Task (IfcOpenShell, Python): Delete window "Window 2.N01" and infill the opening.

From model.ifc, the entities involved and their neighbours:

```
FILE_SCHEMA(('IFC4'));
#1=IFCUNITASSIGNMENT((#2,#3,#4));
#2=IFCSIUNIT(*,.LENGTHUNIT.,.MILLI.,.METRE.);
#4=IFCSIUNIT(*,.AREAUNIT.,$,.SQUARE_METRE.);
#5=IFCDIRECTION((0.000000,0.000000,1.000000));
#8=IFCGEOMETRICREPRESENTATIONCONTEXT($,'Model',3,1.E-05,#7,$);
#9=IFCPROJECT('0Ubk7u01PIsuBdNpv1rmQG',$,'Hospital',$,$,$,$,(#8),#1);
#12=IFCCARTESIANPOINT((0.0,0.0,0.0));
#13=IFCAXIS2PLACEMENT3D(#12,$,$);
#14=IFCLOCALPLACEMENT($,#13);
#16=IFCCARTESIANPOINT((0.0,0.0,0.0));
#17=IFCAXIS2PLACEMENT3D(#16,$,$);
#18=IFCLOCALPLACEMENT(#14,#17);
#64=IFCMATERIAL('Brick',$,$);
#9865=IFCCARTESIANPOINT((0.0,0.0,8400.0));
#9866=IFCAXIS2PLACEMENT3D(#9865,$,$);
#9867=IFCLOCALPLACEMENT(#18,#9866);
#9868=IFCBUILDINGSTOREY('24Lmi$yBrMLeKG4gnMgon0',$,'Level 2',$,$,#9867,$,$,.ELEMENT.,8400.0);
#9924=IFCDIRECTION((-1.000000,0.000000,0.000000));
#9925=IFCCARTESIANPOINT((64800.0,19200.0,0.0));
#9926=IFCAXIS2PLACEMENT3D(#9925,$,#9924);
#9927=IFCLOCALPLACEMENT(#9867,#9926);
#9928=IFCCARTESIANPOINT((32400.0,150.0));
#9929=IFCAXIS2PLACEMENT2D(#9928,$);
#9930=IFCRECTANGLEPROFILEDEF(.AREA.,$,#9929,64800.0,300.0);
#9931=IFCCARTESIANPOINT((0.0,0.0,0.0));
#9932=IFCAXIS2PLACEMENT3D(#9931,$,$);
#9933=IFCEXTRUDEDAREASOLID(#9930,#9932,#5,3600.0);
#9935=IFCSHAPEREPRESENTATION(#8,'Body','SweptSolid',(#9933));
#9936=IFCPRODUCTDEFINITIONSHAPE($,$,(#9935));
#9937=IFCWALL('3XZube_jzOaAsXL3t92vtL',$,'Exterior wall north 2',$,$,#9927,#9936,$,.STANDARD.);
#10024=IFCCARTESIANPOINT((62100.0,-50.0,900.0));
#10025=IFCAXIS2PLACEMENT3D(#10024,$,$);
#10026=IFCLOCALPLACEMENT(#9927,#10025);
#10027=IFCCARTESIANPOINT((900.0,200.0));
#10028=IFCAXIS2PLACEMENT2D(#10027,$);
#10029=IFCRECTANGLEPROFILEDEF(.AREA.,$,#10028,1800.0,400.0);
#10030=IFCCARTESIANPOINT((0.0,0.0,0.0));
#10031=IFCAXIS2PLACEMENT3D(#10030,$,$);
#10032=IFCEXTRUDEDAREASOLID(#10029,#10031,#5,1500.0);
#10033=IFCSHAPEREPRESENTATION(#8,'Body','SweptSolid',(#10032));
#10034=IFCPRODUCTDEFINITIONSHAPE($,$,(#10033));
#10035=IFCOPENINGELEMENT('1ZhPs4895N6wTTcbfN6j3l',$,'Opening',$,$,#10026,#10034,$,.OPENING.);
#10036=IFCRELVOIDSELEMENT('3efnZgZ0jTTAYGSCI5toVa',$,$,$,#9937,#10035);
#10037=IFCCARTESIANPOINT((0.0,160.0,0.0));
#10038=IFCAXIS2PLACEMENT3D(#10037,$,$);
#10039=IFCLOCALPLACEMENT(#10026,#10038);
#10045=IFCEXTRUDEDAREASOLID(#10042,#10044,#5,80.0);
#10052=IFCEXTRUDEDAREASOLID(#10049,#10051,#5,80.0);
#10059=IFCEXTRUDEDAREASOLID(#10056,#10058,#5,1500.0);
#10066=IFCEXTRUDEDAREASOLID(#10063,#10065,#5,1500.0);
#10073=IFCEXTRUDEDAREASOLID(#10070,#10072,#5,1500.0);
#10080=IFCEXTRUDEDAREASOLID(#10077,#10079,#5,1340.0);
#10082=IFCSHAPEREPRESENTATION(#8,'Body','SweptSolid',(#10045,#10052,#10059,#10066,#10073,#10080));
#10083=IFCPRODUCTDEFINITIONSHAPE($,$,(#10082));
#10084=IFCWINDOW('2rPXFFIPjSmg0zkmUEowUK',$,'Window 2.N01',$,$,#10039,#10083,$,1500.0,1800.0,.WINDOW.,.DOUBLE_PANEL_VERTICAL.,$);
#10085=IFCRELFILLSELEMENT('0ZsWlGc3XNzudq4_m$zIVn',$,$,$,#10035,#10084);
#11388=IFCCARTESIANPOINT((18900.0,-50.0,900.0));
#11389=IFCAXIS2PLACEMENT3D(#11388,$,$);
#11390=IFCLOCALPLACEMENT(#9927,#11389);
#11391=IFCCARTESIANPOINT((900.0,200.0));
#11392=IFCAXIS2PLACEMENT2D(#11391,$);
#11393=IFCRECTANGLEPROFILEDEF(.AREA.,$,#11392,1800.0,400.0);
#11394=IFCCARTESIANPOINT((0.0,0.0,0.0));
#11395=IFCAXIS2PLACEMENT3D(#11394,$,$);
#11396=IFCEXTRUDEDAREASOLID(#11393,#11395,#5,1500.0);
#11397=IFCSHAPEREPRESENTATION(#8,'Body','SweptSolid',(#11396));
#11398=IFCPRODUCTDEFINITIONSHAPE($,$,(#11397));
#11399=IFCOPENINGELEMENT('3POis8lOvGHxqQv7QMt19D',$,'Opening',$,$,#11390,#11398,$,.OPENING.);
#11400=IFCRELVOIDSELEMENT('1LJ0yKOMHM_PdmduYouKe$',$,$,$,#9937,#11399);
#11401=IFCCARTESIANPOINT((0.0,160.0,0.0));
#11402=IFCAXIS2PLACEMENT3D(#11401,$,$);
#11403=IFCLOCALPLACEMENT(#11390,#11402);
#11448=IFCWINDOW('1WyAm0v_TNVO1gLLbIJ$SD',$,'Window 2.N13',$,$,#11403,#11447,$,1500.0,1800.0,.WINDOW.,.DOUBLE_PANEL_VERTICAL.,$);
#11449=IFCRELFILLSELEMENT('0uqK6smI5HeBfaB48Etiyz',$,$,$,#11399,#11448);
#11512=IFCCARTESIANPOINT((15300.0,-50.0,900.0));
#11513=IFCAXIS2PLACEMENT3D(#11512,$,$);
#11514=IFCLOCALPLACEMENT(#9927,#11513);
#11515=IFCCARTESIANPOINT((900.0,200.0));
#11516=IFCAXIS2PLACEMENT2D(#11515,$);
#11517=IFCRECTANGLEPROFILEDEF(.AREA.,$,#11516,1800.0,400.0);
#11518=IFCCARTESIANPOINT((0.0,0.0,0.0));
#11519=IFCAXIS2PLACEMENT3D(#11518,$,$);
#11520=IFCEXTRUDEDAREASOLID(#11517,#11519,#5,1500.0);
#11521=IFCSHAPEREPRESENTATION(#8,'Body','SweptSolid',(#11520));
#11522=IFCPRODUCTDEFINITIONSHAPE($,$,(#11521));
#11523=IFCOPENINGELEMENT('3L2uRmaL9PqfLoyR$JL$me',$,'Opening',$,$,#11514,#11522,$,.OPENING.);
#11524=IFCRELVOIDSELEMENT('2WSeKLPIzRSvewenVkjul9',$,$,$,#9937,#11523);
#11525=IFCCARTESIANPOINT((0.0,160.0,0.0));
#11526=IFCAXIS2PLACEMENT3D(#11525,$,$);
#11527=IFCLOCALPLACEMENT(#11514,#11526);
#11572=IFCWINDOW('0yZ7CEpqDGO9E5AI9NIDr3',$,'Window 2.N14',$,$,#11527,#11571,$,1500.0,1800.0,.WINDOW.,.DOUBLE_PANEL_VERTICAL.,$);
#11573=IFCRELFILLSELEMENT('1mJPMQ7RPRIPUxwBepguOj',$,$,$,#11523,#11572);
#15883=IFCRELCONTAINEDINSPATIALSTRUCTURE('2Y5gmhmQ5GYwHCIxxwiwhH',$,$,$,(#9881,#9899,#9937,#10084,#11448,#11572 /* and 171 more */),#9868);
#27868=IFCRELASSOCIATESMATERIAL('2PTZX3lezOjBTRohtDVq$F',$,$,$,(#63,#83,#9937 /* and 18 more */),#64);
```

```python
import ifcopenshell
import ifcopenshell.api.feature
import ifcopenshell.api.root
import ifcopenshell.geom
import ifcopenshell.util.shape

model = ifcopenshell.open("model.ifc")
settings = ifcopenshell.geom.settings()


def volume(element):
    """Net volume in cubic metres, openings subtracted."""
    shape = ifcopenshell.geom.create_shape(settings, element)
    return ifcopenshell.util.shape.get_volume(shape.geometry)


window = model.by_guid("2rPXFFIPjSmg0zkmUEowUK")
opening = window.FillsVoids[0].RelatingOpeningElement
wall = opening.VoidsElements[0].RelatingBuildingElement
before = volume(wall)

ifcopenshell.api.root.remove_product(model, product=window)
ifcopenshell.api.feature.remove_feature(model, feature=opening)

after = volume(wall)

print(f"wall volume {before:.3f} -> {after:.3f} m3")

model.write("model_v2.ifc")
```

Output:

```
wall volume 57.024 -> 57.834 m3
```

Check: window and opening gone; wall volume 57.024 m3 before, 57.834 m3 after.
